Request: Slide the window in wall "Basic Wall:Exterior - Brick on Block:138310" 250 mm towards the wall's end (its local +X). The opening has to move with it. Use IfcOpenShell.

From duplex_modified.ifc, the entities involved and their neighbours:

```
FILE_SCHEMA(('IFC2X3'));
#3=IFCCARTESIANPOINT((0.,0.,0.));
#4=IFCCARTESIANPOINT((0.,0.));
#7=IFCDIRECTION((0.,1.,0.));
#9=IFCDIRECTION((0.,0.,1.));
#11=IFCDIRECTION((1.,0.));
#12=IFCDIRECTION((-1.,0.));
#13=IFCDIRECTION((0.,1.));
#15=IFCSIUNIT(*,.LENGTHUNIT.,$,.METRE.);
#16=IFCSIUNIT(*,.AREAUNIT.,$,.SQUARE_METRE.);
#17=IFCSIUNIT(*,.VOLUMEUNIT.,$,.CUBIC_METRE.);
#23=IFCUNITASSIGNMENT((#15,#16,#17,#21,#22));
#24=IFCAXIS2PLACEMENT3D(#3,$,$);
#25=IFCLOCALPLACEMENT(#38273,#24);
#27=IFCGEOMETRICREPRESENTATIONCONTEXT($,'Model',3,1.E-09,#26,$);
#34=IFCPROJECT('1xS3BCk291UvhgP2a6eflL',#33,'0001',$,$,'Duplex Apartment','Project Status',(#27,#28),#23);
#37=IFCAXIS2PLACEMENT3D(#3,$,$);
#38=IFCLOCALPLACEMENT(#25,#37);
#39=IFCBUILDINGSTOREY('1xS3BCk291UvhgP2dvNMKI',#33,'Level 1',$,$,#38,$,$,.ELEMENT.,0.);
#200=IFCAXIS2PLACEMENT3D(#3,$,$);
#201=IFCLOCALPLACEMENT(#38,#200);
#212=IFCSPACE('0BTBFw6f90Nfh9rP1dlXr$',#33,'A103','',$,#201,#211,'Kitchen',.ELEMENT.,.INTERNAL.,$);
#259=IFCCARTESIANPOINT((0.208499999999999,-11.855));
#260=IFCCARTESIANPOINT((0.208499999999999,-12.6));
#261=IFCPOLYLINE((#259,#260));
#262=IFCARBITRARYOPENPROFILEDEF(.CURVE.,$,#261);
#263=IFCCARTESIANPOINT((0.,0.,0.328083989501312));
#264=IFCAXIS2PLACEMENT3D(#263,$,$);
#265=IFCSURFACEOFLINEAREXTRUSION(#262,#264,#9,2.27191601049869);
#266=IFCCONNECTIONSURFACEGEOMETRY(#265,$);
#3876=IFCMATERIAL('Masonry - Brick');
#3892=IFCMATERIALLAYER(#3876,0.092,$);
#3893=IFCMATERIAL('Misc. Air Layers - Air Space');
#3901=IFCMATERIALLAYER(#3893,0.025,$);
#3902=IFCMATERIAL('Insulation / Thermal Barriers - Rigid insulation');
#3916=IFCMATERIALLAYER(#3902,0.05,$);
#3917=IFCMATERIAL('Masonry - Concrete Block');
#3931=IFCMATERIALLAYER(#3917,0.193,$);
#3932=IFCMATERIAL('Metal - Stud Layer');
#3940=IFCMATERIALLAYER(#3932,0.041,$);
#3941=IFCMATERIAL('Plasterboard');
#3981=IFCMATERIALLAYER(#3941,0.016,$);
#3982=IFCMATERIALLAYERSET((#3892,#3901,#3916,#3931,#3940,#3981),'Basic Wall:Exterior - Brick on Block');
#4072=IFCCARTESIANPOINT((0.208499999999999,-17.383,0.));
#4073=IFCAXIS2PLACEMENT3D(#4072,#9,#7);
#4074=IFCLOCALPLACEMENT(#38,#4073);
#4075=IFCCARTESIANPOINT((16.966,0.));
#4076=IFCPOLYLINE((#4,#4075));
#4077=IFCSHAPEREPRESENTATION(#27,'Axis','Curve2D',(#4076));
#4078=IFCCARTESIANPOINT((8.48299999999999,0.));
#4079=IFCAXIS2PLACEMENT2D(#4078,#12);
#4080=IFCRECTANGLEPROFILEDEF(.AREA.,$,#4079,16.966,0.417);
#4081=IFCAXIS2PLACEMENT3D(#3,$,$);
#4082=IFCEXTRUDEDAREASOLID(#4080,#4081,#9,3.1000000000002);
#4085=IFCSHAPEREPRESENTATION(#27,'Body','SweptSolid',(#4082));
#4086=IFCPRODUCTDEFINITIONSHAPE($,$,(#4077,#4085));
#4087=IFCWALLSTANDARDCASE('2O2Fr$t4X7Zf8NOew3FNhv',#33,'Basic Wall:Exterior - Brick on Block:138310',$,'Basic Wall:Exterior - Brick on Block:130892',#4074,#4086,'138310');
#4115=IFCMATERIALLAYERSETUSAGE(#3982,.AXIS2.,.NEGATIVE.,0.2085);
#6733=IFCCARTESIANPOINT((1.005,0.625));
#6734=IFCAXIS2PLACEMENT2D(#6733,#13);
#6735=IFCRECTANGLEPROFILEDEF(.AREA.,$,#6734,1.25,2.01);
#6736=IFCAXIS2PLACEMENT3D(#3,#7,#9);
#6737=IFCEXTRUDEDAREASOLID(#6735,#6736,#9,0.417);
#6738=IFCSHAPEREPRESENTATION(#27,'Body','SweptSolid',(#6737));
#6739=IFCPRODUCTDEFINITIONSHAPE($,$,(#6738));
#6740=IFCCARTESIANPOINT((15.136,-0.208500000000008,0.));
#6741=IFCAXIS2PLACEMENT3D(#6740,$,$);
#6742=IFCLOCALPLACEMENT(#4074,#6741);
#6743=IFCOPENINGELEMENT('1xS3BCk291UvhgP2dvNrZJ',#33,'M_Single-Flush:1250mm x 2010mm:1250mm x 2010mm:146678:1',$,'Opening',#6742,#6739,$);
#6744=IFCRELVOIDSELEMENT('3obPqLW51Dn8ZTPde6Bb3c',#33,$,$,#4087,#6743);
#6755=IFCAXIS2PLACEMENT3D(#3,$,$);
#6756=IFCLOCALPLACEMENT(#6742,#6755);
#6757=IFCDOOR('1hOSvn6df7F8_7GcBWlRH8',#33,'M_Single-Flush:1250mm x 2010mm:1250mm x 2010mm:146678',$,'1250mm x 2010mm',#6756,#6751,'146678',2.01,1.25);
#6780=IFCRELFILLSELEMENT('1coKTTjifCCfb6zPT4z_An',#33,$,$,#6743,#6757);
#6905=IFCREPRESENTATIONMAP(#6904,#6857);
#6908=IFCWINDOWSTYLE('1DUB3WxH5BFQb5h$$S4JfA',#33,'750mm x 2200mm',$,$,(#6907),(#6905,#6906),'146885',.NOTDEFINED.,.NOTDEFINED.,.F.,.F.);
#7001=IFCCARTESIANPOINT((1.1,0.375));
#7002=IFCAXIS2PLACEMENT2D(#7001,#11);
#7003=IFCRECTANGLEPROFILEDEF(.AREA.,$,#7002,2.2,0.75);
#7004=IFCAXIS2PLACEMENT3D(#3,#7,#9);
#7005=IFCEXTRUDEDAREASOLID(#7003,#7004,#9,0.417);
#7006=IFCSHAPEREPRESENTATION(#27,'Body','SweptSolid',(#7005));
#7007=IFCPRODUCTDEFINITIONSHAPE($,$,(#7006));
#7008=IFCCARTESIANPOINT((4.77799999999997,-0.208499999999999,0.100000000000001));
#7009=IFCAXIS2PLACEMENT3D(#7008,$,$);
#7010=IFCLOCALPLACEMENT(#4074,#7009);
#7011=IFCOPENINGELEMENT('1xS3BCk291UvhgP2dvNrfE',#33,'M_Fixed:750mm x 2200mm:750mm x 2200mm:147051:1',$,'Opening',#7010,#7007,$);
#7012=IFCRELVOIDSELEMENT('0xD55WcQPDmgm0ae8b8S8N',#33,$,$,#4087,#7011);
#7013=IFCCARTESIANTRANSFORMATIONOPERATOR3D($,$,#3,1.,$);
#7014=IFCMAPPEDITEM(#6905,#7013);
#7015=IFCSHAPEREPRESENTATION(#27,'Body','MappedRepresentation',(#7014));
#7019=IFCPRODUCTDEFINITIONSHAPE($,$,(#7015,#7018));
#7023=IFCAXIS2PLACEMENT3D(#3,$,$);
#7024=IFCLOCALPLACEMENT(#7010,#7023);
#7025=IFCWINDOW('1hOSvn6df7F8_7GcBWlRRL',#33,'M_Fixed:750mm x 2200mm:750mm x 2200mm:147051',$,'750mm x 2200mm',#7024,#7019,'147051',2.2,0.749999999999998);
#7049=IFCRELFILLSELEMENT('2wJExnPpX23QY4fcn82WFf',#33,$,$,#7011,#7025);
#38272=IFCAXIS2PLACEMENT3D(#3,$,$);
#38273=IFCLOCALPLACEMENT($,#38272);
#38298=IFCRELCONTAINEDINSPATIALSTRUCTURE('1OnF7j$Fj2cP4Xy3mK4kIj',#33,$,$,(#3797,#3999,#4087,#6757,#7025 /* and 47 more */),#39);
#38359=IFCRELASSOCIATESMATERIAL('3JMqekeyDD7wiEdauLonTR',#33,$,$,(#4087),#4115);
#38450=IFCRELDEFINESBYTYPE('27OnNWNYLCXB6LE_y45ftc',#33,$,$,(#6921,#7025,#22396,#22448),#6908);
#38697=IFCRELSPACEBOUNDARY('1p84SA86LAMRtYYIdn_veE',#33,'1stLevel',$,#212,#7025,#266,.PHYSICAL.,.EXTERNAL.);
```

```python
import numpy as np
import ifcopenshell
import ifcopenshell.api.geometry
import ifcopenshell.util.placement

model = ifcopenshell.open("duplex_modified.ifc")

window = model.by_guid("1hOSvn6df7F8_7GcBWlRRL")
opening = window.FillsVoids[0].RelatingOpeningElement
wall = opening.VoidsElements[0].RelatingBuildingElement

wall_matrix = ifcopenshell.util.placement.get_local_placement(wall.ObjectPlacement)
shift = wall_matrix[:3, 0] * 0.25
before = ifcopenshell.util.placement.get_local_placement(window.ObjectPlacement)[:3, 3].copy()

# The window is placed relative to its opening, so it follows when the opening moves.
matrix = ifcopenshell.util.placement.get_local_placement(opening.ObjectPlacement)
matrix[:3, 3] += shift
ifcopenshell.api.geometry.edit_object_placement(
    model, product=opening, matrix=matrix, is_si=False, should_transform_children=True
)

# Space boundary surfaces are stored in each space's coordinates; move them too.
for rel in window.ProvidesBoundaries:
    if not rel.ConnectionGeometry:
        continue
    surface = rel.ConnectionGeometry.SurfaceOnRelatingElement
    space_matrix = ifcopenshell.util.placement.get_local_placement(rel.RelatingSpace.ObjectPlacement)
    point = np.array(surface.Position.Location.Coordinates) + space_matrix[:3, :3].T @ shift
    surface.Position = model.createIfcAxis2Placement3D(
        model.createIfcCartesianPoint(point.tolist()), surface.Position.Axis, surface.Position.RefDirection
    )

after = ifcopenshell.util.placement.get_local_placement(window.ObjectPlacement)[:3, 3]
print("window moved by", (after - before).round(3) + 0.0)

model.write("duplex_modified_updated.ifc")
```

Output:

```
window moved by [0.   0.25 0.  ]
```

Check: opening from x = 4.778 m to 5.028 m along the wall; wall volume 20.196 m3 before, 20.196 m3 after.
